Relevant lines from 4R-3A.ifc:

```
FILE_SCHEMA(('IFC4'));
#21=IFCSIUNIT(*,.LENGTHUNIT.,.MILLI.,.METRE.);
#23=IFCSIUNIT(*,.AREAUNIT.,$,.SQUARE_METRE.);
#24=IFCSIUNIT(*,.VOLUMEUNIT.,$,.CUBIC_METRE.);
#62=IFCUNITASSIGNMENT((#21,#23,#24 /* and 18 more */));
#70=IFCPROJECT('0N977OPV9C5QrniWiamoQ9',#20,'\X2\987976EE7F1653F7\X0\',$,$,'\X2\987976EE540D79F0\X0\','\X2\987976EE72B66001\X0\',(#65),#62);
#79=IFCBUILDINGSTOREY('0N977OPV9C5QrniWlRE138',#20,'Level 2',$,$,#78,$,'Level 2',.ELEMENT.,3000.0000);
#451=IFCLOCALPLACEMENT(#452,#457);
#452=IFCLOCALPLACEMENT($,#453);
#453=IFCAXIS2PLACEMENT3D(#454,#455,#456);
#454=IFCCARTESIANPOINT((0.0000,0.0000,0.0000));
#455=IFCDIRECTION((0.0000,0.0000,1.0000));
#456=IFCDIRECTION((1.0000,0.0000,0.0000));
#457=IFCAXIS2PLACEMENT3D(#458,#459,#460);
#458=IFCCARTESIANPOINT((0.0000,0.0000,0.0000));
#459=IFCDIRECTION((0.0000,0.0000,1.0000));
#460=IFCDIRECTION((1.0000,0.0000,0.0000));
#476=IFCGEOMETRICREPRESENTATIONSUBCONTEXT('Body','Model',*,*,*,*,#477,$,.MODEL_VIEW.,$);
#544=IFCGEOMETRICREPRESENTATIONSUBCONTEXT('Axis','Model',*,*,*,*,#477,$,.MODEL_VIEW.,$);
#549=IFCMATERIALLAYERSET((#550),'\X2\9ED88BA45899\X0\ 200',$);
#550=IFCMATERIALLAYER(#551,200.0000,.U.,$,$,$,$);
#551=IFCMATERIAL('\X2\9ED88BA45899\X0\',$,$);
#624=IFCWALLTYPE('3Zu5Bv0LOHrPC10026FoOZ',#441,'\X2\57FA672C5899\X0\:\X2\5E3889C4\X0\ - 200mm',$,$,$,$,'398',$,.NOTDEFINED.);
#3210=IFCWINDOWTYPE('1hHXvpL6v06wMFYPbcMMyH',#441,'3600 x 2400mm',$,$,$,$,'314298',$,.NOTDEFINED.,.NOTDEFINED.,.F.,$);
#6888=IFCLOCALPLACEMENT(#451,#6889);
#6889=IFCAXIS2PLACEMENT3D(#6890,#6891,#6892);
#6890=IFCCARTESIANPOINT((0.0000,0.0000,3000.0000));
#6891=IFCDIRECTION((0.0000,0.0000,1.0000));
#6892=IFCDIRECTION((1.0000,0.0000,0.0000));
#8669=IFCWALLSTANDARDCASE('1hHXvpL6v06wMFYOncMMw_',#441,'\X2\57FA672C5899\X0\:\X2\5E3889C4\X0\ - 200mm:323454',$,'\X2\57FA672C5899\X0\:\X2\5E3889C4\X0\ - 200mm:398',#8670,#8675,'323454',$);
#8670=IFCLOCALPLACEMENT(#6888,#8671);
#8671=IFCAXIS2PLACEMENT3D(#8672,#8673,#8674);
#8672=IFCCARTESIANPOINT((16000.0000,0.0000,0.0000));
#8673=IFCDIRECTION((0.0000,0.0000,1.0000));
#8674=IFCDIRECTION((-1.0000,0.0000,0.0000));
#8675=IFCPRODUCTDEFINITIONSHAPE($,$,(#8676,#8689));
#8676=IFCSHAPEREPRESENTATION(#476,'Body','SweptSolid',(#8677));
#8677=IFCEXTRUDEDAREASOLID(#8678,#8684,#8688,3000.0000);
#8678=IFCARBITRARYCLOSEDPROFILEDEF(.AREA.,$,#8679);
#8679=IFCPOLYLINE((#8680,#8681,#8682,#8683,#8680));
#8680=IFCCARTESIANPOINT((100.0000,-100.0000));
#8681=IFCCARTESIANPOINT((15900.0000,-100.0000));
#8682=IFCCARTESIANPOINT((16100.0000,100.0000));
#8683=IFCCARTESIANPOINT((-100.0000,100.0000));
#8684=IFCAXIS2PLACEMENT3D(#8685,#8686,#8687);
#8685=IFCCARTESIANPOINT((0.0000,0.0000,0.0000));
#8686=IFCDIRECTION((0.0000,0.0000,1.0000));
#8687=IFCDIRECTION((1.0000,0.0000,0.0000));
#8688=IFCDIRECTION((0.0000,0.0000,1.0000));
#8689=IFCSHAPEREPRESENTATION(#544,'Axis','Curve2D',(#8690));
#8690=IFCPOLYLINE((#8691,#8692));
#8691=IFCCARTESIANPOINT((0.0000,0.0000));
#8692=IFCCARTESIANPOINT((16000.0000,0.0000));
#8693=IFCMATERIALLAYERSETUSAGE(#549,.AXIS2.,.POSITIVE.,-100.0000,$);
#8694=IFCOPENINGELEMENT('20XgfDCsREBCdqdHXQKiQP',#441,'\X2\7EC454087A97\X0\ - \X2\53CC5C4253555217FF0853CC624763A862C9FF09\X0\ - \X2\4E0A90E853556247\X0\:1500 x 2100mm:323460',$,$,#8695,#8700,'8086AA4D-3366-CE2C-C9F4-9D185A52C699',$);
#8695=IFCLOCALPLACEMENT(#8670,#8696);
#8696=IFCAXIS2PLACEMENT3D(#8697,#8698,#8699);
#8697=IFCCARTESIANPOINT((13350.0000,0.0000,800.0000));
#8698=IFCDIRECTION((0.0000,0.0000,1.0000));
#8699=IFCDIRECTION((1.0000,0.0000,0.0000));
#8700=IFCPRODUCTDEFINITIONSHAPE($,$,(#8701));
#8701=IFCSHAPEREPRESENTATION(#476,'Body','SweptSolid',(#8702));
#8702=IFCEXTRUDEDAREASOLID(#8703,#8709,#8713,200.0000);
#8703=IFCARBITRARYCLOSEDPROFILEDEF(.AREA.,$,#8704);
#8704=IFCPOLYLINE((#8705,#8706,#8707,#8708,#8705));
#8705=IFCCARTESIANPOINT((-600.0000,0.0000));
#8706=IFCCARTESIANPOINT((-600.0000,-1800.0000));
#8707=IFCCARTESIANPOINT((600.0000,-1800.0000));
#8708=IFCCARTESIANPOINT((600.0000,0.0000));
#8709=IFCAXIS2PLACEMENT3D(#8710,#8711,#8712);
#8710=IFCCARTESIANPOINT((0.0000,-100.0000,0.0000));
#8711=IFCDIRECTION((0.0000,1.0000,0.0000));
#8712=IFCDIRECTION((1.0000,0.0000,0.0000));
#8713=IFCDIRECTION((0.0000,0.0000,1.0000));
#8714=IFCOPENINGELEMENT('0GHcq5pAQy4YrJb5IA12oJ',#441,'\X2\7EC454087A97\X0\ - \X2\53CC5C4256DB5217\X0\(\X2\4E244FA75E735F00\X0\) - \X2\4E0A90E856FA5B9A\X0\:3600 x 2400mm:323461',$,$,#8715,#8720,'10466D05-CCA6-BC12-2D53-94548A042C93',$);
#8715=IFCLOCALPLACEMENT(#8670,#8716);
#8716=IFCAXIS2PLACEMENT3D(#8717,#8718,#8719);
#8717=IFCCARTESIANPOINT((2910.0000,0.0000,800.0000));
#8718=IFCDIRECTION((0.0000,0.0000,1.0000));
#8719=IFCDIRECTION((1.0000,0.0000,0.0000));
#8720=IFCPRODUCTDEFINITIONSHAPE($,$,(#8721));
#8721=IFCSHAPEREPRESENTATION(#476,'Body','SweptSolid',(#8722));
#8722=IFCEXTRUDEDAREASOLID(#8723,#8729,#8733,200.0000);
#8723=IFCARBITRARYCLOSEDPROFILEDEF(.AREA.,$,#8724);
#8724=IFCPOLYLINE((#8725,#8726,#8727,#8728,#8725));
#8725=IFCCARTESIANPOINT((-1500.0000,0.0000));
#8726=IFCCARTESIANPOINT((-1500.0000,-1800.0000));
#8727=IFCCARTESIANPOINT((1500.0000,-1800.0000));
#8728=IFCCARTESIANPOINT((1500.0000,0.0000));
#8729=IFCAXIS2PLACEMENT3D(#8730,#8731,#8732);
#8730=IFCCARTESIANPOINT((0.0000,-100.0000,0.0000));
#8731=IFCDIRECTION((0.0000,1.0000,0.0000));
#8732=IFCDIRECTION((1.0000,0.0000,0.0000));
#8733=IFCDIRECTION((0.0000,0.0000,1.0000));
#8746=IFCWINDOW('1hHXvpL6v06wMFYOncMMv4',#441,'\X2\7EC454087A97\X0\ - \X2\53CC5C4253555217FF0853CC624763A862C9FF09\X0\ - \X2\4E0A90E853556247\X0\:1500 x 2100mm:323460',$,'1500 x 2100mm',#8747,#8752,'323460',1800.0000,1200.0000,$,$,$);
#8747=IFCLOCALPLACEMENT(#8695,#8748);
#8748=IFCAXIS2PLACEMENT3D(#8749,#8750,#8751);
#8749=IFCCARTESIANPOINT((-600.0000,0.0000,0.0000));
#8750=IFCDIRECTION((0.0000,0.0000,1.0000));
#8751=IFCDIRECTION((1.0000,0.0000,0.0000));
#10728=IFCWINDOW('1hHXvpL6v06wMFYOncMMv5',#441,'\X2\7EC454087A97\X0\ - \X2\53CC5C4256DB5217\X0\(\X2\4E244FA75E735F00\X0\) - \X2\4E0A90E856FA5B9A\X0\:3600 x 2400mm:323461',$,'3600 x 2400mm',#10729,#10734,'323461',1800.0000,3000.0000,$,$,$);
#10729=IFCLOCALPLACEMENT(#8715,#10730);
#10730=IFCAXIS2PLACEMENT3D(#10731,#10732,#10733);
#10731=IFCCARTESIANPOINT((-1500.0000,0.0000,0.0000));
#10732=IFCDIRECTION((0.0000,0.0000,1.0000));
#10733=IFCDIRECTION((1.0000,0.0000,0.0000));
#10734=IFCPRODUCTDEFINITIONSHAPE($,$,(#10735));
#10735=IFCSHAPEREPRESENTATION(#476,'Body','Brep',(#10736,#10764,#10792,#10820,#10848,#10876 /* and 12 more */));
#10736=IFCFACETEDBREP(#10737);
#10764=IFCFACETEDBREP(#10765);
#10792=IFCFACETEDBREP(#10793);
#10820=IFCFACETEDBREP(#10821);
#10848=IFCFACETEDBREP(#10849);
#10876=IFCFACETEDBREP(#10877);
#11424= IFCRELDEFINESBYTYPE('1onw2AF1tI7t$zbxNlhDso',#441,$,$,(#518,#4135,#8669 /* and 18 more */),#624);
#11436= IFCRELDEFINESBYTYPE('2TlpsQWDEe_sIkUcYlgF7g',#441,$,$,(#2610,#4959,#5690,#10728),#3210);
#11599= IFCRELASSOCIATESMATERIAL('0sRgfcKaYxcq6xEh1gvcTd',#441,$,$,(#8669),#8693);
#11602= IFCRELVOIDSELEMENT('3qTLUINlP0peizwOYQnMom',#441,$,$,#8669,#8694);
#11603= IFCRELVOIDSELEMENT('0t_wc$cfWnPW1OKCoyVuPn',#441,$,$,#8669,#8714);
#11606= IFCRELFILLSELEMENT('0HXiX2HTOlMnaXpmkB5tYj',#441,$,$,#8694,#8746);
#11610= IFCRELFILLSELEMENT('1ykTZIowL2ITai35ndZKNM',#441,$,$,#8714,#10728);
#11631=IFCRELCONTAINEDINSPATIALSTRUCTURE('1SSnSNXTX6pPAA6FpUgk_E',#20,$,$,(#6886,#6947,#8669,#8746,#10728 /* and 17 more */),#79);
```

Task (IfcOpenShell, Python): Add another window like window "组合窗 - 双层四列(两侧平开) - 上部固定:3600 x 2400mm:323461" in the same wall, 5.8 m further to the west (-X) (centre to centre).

```python
import ifcopenshell
import ifcopenshell.api.feature
import ifcopenshell.api.geometry
import ifcopenshell.api.root
import ifcopenshell.geom
import ifcopenshell.util.element
import ifcopenshell.util.placement
import ifcopenshell.util.shape

model = ifcopenshell.open("4R-3A.ifc")
settings = ifcopenshell.geom.settings()


def volume(element):
    """Net volume in cubic metres, openings subtracted."""
    shape = ifcopenshell.geom.create_shape(settings, element)
    return ifcopenshell.util.shape.get_volume(shape.geometry)


def reuse_history(source, copy):
    """copy_class also copies each property set's owner history, people and application; keep the originals."""
    for rel in copy.IsDefinedBy:
        if rel.is_a("IfcRelDefinesByProperties") and (history := rel.RelatingPropertyDefinition.OwnerHistory):
            rel.RelatingPropertyDefinition.OwnerHistory = source.OwnerHistory
            ifcopenshell.util.element.remove_deep2(model, history)


window = model.by_id(10728)
opening = window.FillsVoids[0].RelatingOpeningElement
wall = opening.VoidsElements[0].RelatingBuildingElement
before = volume(wall)
shift = ifcopenshell.util.placement.get_local_placement(wall.ObjectPlacement)[:3, 0] * 5800.0

# copy_class copies the void relationship, type, container and properties, but no geometry.
new_opening = ifcopenshell.api.root.copy_class(model, product=opening)
new_opening.Representation = ifcopenshell.util.element.copy_deep(
    model, opening.Representation, exclude=["IfcGeometricRepresentationContext", "IfcRepresentationMap"]
)
new_opening.Name = "组合窗 - 双层四列(两侧平开) - 上部固定:3600 x 2400mm"
new_opening.Tag = None
new_window = ifcopenshell.api.root.copy_class(model, product=window)
new_window.Representation = ifcopenshell.util.element.copy_deep(
    model, window.Representation, exclude=["IfcGeometricRepresentationContext", "IfcRepresentationMap"]
)
new_window.Name = "组合窗 - 双层四列(两侧平开) - 上部固定:3600 x 2400mm"
new_window.Tag = None
reuse_history(window, new_window)
ifcopenshell.api.feature.add_filling(model, opening=new_opening, element=new_window)

for old, new in ((opening, new_opening), (window, new_window)):
    matrix = ifcopenshell.util.placement.get_local_placement(old.ObjectPlacement)
    matrix[:3, 3] += shift
    ifcopenshell.api.geometry.edit_object_placement(model, product=new, matrix=matrix, is_si=False)

after = volume(wall)

print(f"wall volume {before:.3f} -> {after:.3f} m3")

model.write("4R-3A_edited.ifc")
```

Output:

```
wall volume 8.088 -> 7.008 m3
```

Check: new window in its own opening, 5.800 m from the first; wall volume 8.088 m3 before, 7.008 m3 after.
